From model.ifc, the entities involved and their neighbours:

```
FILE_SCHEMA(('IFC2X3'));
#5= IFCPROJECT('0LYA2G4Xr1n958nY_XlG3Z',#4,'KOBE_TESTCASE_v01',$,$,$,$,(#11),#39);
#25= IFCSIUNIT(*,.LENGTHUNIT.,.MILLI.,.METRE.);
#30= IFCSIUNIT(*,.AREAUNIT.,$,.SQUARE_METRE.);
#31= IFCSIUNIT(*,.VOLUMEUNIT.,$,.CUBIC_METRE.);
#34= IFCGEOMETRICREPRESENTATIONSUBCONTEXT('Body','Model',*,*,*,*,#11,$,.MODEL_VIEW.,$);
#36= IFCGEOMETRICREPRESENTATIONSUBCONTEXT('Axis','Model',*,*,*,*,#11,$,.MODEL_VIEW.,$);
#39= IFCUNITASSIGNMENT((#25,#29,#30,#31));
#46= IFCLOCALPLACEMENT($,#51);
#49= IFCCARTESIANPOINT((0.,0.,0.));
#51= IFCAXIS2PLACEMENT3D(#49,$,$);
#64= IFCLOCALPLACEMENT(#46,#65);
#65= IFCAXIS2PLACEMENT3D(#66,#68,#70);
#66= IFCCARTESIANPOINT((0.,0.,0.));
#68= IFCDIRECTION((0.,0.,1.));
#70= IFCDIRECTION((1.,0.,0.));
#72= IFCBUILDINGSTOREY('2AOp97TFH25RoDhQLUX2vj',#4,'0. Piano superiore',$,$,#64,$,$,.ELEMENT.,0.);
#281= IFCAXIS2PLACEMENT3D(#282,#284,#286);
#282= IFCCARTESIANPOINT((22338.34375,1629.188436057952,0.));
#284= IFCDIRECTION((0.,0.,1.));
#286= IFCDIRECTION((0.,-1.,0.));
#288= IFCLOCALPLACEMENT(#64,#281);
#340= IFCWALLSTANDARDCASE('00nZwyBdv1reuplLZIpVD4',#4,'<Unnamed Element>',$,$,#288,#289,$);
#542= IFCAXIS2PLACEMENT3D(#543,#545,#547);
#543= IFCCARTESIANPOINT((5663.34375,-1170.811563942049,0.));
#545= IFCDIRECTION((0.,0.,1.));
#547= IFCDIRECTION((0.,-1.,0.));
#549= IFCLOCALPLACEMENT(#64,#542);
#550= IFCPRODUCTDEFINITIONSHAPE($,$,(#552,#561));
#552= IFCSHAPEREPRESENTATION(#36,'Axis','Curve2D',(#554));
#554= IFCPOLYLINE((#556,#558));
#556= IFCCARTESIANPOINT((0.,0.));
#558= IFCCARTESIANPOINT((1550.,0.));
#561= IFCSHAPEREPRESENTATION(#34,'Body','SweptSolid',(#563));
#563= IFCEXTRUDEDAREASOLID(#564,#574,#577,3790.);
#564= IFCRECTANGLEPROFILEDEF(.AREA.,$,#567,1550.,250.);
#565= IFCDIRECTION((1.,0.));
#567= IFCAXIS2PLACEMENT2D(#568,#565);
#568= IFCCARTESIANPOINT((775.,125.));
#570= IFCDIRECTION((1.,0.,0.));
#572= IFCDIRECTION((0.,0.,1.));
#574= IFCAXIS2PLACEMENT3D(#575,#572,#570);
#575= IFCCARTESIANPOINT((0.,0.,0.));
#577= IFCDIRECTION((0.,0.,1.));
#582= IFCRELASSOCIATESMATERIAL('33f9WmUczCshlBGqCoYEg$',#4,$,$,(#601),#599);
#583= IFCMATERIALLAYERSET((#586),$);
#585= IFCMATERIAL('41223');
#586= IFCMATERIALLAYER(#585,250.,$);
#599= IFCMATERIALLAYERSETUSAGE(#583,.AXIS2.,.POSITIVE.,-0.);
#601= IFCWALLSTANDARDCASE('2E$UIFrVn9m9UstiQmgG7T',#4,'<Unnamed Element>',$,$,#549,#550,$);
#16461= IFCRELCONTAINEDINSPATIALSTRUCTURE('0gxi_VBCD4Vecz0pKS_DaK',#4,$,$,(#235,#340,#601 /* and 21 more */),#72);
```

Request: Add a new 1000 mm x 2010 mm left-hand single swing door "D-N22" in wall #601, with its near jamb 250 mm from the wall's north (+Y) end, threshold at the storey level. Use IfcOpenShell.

```python
import numpy as np
import ifcopenshell
import ifcopenshell.api.feature
import ifcopenshell.api.geometry
import ifcopenshell.api.root
import ifcopenshell.api.spatial
import ifcopenshell.api.type
import ifcopenshell.geom
import ifcopenshell.util.element
import ifcopenshell.util.placement
import ifcopenshell.util.representation
import ifcopenshell.util.shape
import ifcopenshell.util.unit

model = ifcopenshell.open("model.ifc")
unit_scale = ifcopenshell.util.unit.calculate_unit_scale(model)
settings = ifcopenshell.geom.settings()


def volume(element):
    """Net volume in cubic metres, openings subtracted."""
    shape = ifcopenshell.geom.create_shape(settings, element)
    return ifcopenshell.util.shape.get_volume(shape.geometry)


wall = model.by_guid("2E$UIFrVn9m9UstiQmgG7T")
storey = ifcopenshell.util.element.get_container(wall, ifc_class="IfcBuildingStorey")
context = ifcopenshell.util.representation.get_context(model, "Model", "Body", "MODEL_VIEW")
before = volume(wall)

width, height, from_end, sill = 1, 2.01, 0.25, 0.0  # metres

# The wall runs along its own X axis, and the end named is its -X end.
wall_shape = ifcopenshell.geom.create_shape(settings, wall)
x, y, z = ifcopenshell.util.shape.get_vertices(wall_shape.geometry).T
start = x.min() + from_end
face, thickness = float(y.min()), float(y.max() - y.min())
wall_matrix = ifcopenshell.util.placement.get_local_placement(wall.ObjectPlacement)
level = ifcopenshell.util.placement.get_local_placement(storey.ObjectPlacement)[2, 3]


def in_wall(x, y):
    """Placement at x, y metres in the wall's axes, at sill height."""
    matrix = wall_matrix.copy()
    matrix[:, 3] = wall_matrix @ np.array([x / unit_scale, y / unit_scale, 0.0, 1.0])
    matrix[2, 3] = level + sill / unit_scale
    return matrix


# Opening: a box that overshoots both wall faces by 50 mm.
opening = ifcopenshell.api.root.create_entity(model, ifc_class="IfcOpeningElement")
box = ifcopenshell.api.geometry.add_wall_representation(
    model, context=context, length=width, height=height, thickness=thickness + 0.1
)
ifcopenshell.api.geometry.assign_representation(model, product=opening, representation=box)
ifcopenshell.api.geometry.edit_object_placement(model, product=opening, matrix=in_wall(start, face - 0.05), is_si=False)
ifcopenshell.api.feature.add_feature(model, feature=opening, element=wall)

door = ifcopenshell.api.root.create_entity(model, ifc_class="IfcDoor", name="D-N22")
door.OverallWidth, door.OverallHeight = width / unit_scale, height / unit_scale
body = ifcopenshell.api.geometry.add_door_representation(
    model,
    context=context,
    overall_width=door.OverallWidth,
    overall_height=door.OverallHeight,
    operation_type="SINGLE_SWING_LEFT",
    lining_properties={"LiningDepth": thickness / unit_scale, "ThresholdDepth": thickness / unit_scale},
)
ifcopenshell.api.geometry.assign_representation(model, product=door, representation=body)
ifcopenshell.api.spatial.assign_container(model, products=[door], relating_structure=storey)
fills = ifcopenshell.api.feature.add_filling(model, opening=opening, element=door)
fills.OwnerHistory = door.OwnerHistory  # required in IFC2X3

# IFC2X3 keeps the operation on the door style.
style = ifcopenshell.api.root.create_entity(model, ifc_class="IfcDoorStyle", name="D-N22")
style.OperationType, style.ConstructionType = "SINGLE_SWING_LEFT", "NOTDEFINED"
style.ParameterTakesPrecedence = style.Sizeable = False
ifcopenshell.api.type.assign_type(model, related_objects=[door], relating_type=style)

# The lining spans the wall, so the door starts at the wall face.
ifcopenshell.api.geometry.edit_object_placement(model, product=door, matrix=in_wall(start, face), is_si=False)

after = volume(wall)

print(f"wall volume {before:.3f} -> {after:.3f} m3")

model.write("model_rev.ifc")
```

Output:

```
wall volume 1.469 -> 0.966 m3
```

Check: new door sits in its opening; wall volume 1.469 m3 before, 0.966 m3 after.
